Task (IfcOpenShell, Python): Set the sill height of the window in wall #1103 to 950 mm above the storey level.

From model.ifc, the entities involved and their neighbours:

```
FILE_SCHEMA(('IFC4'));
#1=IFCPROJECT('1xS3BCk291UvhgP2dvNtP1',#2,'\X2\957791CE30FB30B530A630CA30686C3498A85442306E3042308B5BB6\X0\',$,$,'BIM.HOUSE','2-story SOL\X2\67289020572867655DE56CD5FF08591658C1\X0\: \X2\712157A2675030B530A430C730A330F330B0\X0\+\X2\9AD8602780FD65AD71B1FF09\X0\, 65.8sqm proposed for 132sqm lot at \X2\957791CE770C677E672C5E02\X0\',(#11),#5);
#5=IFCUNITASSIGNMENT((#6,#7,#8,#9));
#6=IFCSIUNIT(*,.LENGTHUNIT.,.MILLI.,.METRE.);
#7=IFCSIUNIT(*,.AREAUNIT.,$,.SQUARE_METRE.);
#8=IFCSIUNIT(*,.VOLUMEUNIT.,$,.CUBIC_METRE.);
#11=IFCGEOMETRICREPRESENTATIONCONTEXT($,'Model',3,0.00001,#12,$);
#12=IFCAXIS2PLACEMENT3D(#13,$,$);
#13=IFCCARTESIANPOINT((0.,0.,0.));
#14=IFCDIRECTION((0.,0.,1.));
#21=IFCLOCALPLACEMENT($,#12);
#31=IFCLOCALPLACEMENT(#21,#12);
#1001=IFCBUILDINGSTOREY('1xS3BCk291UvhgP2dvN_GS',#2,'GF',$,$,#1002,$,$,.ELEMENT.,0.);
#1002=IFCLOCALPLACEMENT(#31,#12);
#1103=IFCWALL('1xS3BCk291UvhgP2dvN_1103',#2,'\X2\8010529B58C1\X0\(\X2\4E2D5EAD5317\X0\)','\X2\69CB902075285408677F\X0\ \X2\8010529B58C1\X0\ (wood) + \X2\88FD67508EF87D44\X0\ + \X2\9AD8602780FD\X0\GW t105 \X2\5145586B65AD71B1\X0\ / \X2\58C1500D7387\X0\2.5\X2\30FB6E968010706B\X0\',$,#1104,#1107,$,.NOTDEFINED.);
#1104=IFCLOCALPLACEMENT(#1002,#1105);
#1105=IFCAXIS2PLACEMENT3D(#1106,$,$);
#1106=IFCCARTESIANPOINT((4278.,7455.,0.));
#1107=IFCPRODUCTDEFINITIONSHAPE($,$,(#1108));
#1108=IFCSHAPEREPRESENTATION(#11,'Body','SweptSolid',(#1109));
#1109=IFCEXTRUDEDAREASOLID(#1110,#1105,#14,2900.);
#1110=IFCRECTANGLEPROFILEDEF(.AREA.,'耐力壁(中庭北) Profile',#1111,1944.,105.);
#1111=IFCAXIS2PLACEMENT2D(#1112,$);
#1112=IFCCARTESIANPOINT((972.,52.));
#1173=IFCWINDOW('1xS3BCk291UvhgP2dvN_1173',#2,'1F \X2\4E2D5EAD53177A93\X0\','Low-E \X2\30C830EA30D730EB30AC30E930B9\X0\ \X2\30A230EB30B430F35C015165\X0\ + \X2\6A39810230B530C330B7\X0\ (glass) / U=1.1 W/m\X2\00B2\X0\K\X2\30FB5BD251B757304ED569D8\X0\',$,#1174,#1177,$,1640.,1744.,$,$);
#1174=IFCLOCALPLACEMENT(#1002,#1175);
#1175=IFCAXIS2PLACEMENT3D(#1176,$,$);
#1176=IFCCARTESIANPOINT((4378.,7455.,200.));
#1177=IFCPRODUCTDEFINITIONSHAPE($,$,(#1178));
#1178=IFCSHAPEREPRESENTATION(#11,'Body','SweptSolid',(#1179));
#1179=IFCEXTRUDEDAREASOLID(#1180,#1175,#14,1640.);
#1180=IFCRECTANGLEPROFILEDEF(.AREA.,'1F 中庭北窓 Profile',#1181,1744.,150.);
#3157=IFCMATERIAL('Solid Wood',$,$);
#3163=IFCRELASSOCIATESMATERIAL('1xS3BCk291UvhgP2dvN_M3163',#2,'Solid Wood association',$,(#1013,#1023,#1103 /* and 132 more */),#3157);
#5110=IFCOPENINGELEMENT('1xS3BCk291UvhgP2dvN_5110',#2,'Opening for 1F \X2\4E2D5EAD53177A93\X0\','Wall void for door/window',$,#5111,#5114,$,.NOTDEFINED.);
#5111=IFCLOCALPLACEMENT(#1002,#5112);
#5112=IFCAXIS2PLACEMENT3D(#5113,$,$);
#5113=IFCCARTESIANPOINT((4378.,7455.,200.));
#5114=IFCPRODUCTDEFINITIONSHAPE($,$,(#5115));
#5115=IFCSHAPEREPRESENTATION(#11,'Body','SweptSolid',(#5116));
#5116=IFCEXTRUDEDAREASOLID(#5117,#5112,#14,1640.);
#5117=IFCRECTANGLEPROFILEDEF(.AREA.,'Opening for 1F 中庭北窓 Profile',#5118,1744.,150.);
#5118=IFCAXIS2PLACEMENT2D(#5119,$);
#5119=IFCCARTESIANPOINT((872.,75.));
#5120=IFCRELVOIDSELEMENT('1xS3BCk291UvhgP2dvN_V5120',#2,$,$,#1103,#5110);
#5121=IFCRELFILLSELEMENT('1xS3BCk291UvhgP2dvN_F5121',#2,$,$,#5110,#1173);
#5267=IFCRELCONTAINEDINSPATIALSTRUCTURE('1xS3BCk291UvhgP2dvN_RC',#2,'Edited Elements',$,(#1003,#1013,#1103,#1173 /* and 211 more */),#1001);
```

```python
import numpy as np
import ifcopenshell
import ifcopenshell.api.geometry
import ifcopenshell.geom
import ifcopenshell.util.element
import ifcopenshell.util.placement
import ifcopenshell.util.shape
import ifcopenshell.util.unit

model = ifcopenshell.open("model.ifc")
unit_scale = ifcopenshell.util.unit.calculate_unit_scale(model)

window = model.by_guid("1xS3BCk291UvhgP2dvN_1173")
opening = window.FillsVoids[0].RelatingOpeningElement
storey = ifcopenshell.util.element.get_container(window, ifc_class="IfcBuildingStorey")
level = ifcopenshell.util.placement.get_local_placement(storey.ObjectPlacement)[2, 3]

# The opening's origin need not be at the sill, so measure its lowest point.
shape = ifcopenshell.geom.create_shape(ifcopenshell.geom.settings(), opening)
bottom = ifcopenshell.util.shape.get_shape_bottom_elevation(shape, shape.geometry) / unit_scale
dz = level + 0.95 / unit_scale - bottom

shift = np.array([0.0, 0.0, dz])
# The window is not placed relative to its opening, so move both.
for product in (opening, window):
    matrix = ifcopenshell.util.placement.get_local_placement(product.ObjectPlacement)
    matrix[:3, 3] += shift
    ifcopenshell.api.geometry.edit_object_placement(model, product=product, matrix=matrix, is_si=False)

print(f"moved by {dz * unit_scale:+.3f} m")

model.write("model_v2.ifc")
```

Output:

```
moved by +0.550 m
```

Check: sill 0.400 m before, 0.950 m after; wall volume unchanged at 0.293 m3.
